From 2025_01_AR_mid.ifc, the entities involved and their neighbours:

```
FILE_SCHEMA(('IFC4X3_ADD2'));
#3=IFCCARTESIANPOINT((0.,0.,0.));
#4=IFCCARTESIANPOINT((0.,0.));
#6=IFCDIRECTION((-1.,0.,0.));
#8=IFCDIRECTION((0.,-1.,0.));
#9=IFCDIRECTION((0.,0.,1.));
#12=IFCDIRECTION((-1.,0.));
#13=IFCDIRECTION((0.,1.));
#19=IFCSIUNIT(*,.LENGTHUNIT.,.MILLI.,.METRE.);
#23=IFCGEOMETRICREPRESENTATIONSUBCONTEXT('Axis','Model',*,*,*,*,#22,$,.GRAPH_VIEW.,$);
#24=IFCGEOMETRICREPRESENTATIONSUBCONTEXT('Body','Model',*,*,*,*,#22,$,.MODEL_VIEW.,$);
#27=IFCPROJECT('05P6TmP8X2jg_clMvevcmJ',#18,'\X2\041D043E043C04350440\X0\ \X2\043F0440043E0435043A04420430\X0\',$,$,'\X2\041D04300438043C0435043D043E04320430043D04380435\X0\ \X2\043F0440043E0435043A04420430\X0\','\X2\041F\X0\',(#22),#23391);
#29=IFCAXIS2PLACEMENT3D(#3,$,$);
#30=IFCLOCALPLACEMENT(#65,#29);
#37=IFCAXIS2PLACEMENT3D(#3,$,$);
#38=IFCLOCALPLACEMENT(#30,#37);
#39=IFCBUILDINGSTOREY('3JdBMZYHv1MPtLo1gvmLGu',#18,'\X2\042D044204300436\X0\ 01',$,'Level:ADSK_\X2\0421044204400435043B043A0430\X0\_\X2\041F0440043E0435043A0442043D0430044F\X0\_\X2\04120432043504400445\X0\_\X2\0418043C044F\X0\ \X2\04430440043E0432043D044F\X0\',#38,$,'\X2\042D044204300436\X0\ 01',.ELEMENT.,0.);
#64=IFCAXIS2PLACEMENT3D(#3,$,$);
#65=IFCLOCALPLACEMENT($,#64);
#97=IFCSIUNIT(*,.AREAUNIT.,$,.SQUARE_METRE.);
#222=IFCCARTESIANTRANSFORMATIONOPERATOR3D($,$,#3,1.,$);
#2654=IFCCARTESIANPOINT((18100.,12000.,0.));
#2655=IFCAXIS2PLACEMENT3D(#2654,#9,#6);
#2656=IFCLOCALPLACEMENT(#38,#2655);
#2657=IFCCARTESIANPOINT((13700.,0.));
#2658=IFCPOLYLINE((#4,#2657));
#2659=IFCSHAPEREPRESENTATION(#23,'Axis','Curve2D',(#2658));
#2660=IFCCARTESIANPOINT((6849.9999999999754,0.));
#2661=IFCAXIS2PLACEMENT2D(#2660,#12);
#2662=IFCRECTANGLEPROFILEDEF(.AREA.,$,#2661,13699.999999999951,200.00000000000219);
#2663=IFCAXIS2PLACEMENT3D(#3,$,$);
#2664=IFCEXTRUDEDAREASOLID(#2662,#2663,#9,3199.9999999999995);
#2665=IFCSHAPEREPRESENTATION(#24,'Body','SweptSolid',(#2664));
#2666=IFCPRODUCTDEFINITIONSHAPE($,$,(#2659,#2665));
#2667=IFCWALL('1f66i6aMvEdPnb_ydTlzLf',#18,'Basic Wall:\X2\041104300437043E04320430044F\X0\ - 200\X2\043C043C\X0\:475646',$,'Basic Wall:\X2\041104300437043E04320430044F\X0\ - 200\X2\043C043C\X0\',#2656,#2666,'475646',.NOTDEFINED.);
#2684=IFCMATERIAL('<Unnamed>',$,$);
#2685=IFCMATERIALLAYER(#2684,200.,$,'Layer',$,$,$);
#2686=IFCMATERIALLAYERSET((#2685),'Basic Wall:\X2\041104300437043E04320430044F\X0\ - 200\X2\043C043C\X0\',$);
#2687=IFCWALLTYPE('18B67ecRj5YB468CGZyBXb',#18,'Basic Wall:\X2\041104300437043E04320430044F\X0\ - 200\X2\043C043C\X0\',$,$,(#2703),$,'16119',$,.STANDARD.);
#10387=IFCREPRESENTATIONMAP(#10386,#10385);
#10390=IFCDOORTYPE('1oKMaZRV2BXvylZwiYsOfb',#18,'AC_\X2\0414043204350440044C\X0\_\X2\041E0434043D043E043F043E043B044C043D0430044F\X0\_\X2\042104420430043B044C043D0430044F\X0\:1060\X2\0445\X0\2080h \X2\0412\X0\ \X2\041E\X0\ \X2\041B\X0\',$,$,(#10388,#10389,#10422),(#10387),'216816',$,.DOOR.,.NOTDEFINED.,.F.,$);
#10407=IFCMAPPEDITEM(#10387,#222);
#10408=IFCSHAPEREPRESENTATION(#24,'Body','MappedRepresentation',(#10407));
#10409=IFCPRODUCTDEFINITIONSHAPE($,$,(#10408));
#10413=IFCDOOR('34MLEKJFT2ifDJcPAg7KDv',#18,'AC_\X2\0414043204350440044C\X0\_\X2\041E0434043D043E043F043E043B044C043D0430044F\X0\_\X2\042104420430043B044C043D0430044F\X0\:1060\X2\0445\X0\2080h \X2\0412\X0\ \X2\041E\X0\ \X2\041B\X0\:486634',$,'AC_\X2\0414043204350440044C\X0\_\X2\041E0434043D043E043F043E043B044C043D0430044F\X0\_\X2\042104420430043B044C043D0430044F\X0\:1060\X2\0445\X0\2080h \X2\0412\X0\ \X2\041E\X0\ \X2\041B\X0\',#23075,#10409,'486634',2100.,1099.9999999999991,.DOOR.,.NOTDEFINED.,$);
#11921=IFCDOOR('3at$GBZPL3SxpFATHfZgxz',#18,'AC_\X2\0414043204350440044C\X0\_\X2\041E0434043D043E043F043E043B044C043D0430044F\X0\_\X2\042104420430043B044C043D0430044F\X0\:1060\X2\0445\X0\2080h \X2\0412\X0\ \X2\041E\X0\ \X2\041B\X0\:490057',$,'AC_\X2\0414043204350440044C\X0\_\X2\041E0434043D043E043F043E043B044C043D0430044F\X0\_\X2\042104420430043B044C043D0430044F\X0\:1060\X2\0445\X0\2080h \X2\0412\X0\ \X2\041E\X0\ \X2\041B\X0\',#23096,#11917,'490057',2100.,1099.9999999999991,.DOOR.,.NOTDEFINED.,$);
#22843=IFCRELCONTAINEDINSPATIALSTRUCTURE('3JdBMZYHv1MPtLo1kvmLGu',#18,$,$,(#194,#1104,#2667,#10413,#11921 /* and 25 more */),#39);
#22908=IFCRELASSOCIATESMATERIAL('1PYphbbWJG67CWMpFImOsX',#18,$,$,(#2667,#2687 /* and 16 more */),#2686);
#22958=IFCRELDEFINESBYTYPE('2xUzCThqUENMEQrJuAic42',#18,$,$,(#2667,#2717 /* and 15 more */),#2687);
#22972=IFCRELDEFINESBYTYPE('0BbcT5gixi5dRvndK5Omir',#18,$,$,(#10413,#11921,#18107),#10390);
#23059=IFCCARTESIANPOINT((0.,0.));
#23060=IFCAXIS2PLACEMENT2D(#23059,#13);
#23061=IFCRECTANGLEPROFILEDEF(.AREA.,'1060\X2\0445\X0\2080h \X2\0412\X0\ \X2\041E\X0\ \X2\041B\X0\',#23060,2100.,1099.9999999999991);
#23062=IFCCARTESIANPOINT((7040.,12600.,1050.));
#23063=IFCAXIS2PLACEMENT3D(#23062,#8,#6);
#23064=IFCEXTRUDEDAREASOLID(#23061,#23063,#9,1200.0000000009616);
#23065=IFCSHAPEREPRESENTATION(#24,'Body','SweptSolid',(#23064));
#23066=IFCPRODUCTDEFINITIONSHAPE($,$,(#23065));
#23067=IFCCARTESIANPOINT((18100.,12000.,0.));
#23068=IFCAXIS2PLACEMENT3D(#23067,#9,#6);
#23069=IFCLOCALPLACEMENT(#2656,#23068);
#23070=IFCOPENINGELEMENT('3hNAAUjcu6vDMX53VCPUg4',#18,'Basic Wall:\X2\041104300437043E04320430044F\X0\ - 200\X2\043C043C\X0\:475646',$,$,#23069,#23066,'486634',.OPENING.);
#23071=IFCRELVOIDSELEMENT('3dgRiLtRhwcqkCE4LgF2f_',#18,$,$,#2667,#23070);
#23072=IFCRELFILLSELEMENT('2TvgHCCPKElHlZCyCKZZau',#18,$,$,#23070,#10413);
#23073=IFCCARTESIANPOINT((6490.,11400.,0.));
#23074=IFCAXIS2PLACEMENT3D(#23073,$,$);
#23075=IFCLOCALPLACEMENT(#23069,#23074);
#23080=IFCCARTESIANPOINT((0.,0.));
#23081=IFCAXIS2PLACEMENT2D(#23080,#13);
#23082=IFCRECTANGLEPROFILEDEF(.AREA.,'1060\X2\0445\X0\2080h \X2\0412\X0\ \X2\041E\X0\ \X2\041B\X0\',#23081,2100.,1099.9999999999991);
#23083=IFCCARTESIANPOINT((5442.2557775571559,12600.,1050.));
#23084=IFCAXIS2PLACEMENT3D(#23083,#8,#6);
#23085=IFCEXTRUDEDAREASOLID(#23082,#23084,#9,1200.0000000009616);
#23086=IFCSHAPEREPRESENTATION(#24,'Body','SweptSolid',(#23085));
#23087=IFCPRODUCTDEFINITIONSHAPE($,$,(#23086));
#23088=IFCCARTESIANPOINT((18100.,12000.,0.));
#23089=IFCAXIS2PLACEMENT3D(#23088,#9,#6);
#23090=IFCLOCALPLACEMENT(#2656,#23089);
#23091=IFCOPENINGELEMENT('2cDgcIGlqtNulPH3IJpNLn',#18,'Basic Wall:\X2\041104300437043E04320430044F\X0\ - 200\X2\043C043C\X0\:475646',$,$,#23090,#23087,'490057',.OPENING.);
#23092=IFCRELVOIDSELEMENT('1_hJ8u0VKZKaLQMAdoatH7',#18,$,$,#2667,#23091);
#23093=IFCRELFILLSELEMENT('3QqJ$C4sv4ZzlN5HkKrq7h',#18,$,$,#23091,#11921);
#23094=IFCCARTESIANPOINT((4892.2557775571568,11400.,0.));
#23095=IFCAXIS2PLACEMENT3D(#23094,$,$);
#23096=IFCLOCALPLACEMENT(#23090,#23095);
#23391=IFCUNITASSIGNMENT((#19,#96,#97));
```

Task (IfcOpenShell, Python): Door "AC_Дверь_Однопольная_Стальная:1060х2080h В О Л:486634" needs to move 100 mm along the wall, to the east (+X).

```python
import ifcopenshell
import ifcopenshell.api.geometry
import ifcopenshell.util.placement

model = ifcopenshell.open("2025_01_AR_mid.ifc")

door = model.by_guid("34MLEKJFT2ifDJcPAg7KDv")
opening = door.FillsVoids[0].RelatingOpeningElement
wall = opening.VoidsElements[0].RelatingBuildingElement

wall_matrix = ifcopenshell.util.placement.get_local_placement(wall.ObjectPlacement)
shift = wall_matrix[:3, 0] * -100.0
before = ifcopenshell.util.placement.get_local_placement(door.ObjectPlacement)[:3, 3].copy()

# The door is placed relative to its opening, so it follows when the opening moves.
matrix = ifcopenshell.util.placement.get_local_placement(opening.ObjectPlacement)
matrix[:3, 3] += shift
ifcopenshell.api.geometry.edit_object_placement(
    model, product=opening, matrix=matrix, is_si=False, should_transform_children=True
)

after = ifcopenshell.util.placement.get_local_placement(door.ObjectPlacement)[:3, 3]
print("door moved by", (after - before).round(3) + 0.0)

model.write("2025_01_AR_mid-out.ifc")
```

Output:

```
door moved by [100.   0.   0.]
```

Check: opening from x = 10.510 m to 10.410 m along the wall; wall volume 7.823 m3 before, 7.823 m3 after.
